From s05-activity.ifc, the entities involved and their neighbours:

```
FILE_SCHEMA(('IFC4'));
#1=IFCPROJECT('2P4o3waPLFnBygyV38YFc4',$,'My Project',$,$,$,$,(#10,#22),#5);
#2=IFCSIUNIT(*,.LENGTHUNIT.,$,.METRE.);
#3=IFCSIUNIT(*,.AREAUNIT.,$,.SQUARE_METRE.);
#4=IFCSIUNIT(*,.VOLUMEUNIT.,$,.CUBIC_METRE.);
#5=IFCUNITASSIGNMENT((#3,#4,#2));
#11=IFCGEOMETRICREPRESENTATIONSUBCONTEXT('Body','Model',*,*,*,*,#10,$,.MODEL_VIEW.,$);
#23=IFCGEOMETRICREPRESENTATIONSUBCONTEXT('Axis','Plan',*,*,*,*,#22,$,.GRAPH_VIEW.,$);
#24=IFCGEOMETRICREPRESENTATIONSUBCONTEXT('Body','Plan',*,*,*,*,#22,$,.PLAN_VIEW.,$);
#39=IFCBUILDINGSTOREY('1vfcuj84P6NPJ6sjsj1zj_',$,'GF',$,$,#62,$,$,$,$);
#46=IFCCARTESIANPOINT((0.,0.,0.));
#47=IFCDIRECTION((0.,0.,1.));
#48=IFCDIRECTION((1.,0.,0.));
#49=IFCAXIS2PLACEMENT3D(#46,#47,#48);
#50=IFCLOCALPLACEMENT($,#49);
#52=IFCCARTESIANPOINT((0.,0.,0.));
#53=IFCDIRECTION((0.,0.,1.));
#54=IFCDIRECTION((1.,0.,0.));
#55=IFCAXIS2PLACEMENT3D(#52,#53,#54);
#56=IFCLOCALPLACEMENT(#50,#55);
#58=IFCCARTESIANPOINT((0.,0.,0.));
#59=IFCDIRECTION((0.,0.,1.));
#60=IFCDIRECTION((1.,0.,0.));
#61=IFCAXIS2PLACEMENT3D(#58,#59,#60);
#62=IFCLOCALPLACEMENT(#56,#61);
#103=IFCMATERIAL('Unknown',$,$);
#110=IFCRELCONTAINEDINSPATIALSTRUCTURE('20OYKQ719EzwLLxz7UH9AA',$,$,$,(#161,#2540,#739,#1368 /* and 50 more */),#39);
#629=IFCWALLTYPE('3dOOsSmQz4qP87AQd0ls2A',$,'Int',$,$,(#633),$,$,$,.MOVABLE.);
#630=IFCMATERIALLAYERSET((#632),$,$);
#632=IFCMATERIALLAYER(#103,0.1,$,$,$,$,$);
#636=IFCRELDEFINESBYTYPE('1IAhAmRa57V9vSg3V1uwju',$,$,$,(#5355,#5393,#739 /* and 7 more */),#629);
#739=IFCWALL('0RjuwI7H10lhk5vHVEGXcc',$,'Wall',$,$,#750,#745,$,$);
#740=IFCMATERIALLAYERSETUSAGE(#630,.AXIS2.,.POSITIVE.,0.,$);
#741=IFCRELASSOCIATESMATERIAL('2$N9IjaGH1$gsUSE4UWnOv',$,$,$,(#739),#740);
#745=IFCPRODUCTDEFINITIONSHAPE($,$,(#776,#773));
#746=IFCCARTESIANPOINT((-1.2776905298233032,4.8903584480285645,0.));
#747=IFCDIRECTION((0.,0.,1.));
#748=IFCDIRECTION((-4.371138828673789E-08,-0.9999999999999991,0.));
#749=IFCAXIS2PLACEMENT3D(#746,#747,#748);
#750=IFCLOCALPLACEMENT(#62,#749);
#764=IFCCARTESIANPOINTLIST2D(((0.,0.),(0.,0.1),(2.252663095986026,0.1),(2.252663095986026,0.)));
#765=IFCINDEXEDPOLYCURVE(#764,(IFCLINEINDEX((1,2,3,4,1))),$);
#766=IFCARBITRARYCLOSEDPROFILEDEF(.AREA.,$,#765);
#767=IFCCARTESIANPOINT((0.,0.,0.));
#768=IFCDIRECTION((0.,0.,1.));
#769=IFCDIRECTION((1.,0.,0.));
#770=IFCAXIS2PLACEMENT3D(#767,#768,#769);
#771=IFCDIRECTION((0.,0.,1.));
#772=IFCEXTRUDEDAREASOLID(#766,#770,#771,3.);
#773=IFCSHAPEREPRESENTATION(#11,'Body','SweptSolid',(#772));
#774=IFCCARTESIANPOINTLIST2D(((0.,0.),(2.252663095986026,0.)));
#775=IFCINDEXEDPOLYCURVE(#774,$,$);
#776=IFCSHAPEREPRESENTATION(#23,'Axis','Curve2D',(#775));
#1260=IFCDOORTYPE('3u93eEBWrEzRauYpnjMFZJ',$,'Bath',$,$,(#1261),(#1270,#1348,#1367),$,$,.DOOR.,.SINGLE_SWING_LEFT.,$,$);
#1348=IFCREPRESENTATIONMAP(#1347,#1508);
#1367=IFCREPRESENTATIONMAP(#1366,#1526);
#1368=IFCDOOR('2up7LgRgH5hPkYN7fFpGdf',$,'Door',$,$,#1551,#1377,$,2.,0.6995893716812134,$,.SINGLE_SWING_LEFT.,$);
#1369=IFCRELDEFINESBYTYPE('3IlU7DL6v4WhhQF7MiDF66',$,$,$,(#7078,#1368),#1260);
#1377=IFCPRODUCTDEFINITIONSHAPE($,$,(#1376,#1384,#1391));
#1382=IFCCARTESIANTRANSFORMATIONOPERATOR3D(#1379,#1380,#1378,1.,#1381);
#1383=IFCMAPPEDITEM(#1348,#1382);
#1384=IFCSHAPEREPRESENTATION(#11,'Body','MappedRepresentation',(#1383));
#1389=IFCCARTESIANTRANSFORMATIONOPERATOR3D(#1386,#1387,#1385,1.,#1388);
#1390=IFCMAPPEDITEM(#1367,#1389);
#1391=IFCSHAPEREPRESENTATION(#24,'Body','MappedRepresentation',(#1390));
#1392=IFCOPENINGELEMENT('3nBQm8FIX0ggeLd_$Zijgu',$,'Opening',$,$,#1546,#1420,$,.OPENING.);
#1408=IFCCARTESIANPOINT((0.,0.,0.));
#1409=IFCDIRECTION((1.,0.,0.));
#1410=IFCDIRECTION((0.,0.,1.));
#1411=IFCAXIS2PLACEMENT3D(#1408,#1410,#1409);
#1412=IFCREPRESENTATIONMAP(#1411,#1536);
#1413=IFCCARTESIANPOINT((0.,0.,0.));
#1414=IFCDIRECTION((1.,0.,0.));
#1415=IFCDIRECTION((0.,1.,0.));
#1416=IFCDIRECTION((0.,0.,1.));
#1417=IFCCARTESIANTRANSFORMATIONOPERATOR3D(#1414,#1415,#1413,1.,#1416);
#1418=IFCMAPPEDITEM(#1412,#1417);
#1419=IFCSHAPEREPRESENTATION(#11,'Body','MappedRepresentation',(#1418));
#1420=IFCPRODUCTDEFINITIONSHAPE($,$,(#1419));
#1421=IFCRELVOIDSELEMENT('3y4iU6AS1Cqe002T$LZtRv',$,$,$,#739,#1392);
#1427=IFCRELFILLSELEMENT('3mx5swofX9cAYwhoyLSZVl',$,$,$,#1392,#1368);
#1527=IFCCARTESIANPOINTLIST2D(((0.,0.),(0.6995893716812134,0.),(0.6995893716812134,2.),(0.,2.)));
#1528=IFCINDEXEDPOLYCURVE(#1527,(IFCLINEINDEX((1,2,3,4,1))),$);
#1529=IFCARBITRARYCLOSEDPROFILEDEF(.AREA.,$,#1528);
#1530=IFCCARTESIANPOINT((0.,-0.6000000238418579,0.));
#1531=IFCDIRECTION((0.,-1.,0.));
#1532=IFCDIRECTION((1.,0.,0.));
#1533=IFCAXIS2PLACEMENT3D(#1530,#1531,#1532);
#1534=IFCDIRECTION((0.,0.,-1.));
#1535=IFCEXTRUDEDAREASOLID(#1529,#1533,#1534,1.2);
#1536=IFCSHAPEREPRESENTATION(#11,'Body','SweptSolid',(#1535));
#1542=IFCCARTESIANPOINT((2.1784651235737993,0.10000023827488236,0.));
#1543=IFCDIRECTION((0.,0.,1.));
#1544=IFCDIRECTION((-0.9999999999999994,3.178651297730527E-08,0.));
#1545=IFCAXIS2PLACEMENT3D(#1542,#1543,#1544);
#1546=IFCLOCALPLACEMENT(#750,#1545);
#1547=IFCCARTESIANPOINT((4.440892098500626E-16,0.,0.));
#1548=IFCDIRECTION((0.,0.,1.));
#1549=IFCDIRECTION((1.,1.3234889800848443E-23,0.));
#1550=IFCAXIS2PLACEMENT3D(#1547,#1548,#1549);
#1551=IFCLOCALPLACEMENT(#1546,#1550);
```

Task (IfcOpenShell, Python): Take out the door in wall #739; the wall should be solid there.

```python
import ifcopenshell
import ifcopenshell.api.feature
import ifcopenshell.api.root
import ifcopenshell.geom
import ifcopenshell.util.shape

model = ifcopenshell.open("s05-activity.ifc")
settings = ifcopenshell.geom.settings()


def volume(element):
    """Net volume in cubic metres, openings subtracted."""
    shape = ifcopenshell.geom.create_shape(settings, element)
    return ifcopenshell.util.shape.get_volume(shape.geometry)


door = model.by_guid("2up7LgRgH5hPkYN7fFpGdf")
opening = door.FillsVoids[0].RelatingOpeningElement
wall = opening.VoidsElements[0].RelatingBuildingElement
before = volume(wall)

ifcopenshell.api.root.remove_product(model, product=door)
ifcopenshell.api.feature.remove_feature(model, feature=opening)

after = volume(wall)

print(f"wall volume {before:.3f} -> {after:.3f} m3")

model.write("s05-activity_v2.ifc")
```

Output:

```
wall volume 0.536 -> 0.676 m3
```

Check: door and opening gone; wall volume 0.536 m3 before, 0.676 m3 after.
